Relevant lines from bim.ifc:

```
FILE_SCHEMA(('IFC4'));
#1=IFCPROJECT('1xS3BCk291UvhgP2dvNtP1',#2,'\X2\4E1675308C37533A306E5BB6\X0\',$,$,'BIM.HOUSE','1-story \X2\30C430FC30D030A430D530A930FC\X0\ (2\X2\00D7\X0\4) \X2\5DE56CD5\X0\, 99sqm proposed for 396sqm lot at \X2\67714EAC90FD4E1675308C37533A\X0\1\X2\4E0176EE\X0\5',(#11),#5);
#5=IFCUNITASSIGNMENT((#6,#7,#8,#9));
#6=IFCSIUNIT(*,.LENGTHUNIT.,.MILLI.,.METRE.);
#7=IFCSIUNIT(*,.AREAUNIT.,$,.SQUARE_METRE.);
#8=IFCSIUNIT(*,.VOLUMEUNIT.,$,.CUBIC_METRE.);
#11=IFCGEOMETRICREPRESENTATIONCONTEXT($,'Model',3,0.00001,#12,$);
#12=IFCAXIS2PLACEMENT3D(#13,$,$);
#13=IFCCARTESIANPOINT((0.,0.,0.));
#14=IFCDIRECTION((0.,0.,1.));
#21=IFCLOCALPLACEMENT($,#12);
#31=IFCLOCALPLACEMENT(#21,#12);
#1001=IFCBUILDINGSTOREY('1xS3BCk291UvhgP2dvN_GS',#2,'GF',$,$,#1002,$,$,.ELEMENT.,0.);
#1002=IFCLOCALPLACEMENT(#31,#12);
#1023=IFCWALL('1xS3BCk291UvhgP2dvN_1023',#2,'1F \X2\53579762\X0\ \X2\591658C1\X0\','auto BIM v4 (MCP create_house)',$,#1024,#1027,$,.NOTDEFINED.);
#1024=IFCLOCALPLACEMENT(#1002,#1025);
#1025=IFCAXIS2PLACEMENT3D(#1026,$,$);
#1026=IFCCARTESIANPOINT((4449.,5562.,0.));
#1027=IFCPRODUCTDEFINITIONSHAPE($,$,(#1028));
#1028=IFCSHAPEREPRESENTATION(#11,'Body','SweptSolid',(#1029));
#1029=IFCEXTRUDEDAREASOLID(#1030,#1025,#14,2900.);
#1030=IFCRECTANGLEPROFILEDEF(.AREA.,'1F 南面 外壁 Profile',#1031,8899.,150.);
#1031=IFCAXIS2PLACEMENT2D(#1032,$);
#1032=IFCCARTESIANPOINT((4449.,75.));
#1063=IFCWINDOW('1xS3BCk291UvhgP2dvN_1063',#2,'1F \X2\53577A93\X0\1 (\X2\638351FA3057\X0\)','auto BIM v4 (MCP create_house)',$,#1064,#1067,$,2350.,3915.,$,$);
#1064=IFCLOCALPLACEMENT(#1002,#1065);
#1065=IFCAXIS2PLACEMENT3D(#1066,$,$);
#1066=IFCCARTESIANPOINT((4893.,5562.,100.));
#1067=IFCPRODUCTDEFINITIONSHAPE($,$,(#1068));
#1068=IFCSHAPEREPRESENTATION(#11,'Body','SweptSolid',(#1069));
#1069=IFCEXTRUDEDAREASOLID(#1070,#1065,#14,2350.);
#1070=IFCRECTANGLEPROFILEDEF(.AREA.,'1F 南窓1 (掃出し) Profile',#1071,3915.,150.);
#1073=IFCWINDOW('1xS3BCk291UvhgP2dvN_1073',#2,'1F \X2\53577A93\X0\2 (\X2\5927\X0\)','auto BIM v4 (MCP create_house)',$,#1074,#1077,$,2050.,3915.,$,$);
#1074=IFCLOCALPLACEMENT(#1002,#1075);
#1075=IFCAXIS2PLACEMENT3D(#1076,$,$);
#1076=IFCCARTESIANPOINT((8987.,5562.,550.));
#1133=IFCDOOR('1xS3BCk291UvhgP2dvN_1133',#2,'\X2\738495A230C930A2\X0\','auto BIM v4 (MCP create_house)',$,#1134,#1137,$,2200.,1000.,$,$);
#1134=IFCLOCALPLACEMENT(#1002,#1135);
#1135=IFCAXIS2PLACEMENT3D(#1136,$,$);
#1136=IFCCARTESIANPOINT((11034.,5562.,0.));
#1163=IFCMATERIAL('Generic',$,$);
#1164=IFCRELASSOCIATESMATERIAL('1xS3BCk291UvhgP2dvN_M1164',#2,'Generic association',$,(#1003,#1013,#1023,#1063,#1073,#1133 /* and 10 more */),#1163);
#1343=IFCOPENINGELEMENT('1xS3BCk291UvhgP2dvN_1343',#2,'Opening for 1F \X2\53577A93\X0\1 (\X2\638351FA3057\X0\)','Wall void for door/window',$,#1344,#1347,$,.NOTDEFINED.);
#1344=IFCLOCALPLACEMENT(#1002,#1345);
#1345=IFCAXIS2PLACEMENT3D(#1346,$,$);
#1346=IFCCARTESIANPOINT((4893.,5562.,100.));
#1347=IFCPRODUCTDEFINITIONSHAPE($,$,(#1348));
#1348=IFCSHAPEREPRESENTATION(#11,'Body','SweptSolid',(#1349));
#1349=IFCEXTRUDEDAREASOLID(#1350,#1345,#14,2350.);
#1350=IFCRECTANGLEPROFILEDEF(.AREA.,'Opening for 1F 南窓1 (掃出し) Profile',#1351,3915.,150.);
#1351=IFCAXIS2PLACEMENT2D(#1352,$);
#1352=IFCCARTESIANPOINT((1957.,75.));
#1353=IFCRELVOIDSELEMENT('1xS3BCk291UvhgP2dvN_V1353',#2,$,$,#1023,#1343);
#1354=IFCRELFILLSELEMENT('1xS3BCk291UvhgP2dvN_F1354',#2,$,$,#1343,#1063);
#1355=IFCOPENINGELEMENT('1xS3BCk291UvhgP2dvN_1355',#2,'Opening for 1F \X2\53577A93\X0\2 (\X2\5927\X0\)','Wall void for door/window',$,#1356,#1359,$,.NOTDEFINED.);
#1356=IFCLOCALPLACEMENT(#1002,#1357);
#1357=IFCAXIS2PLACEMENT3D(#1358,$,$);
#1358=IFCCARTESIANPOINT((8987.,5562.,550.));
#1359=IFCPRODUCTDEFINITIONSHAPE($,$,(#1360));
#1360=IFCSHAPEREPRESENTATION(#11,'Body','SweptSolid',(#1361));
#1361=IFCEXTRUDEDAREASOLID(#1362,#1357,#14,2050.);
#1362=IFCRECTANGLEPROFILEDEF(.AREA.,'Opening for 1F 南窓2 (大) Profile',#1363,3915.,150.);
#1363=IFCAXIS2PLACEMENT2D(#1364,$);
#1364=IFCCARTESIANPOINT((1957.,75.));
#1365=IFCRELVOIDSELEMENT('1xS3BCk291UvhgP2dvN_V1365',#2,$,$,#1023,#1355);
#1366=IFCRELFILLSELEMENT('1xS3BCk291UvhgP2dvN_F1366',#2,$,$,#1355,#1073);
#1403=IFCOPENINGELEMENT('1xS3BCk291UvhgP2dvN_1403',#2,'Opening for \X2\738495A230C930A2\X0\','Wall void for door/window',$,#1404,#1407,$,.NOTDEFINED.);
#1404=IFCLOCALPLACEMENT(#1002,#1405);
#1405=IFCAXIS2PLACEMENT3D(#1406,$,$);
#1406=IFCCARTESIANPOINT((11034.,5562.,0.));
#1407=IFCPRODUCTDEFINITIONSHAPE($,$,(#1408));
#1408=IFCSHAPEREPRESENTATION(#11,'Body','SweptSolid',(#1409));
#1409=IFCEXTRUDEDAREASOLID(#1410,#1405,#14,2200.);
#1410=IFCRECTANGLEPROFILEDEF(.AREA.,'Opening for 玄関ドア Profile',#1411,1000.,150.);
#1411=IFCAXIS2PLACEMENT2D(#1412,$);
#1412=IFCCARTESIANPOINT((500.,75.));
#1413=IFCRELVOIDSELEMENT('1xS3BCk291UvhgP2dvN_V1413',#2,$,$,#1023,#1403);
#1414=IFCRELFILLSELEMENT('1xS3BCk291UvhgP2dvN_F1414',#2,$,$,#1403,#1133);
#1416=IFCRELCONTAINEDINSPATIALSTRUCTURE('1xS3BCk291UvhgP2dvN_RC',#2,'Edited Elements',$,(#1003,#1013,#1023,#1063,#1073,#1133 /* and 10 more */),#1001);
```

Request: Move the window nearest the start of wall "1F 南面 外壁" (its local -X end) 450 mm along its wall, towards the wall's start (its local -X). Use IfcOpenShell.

```python
import ifcopenshell
import ifcopenshell.api.geometry
import ifcopenshell.util.placement
import ifcopenshell.util.unit

model = ifcopenshell.open("bim.ifc")
unit_scale = ifcopenshell.util.unit.calculate_unit_scale(model)

window = model.by_guid("1xS3BCk291UvhgP2dvN_1063")
opening = window.FillsVoids[0].RelatingOpeningElement
wall = opening.VoidsElements[0].RelatingBuildingElement

wall_matrix = ifcopenshell.util.placement.get_local_placement(wall.ObjectPlacement)
shift = wall_matrix[:3, 0] * -0.45 / unit_scale
before = ifcopenshell.util.placement.get_local_placement(window.ObjectPlacement)[:3, 3].copy()

# The window is not placed relative to its opening, so move both.
for product in (opening, window):
    matrix = ifcopenshell.util.placement.get_local_placement(product.ObjectPlacement)
    matrix[:3, 3] += shift
    ifcopenshell.api.geometry.edit_object_placement(model, product=product, matrix=matrix, is_si=False)

after = ifcopenshell.util.placement.get_local_placement(window.ObjectPlacement)[:3, 3]
print("window moved by", (after - before).round(3) + 0.0)

model.write("bim_v2.ifc")
```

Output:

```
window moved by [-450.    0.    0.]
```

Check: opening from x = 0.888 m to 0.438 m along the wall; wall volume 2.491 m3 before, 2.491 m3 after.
